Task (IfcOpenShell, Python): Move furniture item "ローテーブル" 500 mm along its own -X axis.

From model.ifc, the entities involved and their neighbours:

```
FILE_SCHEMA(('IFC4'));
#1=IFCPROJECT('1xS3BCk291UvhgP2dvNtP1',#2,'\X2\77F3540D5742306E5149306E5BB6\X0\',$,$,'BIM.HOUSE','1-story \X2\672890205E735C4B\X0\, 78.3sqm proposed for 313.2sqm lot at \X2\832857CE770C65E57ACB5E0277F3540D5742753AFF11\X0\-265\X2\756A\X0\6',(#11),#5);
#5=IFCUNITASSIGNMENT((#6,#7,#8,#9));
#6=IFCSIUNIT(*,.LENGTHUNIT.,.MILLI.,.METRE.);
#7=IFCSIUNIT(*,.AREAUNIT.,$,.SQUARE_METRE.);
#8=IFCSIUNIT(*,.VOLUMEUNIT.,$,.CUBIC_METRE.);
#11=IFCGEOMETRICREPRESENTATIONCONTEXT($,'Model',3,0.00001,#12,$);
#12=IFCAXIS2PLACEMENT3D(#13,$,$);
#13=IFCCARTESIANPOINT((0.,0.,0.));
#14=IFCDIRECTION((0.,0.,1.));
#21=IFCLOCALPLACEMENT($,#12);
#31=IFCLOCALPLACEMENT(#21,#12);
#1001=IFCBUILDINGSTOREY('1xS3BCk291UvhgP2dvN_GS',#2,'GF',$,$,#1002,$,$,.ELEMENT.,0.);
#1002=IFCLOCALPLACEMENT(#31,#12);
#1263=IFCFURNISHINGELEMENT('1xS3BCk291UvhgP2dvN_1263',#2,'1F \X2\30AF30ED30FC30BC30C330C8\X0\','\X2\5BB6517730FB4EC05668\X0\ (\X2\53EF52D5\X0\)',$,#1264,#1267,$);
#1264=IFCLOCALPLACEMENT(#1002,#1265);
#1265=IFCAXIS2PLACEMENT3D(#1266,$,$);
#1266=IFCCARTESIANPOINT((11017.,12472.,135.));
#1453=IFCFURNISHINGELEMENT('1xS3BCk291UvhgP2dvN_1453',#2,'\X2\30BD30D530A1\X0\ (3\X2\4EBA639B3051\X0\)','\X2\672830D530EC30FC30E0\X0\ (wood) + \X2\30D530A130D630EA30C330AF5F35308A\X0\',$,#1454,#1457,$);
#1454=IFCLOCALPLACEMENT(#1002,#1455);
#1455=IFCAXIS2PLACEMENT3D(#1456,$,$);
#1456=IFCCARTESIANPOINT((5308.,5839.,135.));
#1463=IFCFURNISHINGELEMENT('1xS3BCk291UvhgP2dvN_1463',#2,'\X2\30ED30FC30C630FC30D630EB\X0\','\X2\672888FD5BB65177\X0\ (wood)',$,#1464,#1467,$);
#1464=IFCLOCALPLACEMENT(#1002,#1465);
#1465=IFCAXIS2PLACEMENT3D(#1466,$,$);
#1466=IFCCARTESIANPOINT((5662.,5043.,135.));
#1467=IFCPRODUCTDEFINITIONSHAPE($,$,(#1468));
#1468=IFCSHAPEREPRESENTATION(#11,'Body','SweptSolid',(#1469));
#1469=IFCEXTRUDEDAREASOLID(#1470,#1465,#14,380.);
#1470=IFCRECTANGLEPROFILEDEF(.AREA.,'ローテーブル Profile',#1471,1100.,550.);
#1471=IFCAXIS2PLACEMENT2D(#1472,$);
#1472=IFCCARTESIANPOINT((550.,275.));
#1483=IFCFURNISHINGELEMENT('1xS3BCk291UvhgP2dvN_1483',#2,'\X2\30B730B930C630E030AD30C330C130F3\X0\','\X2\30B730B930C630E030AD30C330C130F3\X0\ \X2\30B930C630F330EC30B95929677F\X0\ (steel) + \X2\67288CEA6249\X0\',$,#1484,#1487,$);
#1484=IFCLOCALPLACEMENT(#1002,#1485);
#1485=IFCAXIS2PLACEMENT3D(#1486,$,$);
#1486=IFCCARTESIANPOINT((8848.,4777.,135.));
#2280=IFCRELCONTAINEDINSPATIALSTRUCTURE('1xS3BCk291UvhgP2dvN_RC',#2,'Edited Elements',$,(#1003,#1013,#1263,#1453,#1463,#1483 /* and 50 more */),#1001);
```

```python
import ifcopenshell
import ifcopenshell.api.geometry
import ifcopenshell.util.placement
import ifcopenshell.util.unit

model = ifcopenshell.open("model.ifc")
unit_scale = ifcopenshell.util.unit.calculate_unit_scale(model)

item = model.by_guid("1xS3BCk291UvhgP2dvN_1463")
matrix = ifcopenshell.util.placement.get_local_placement(item.ObjectPlacement)
matrix[:3, 3] -= matrix[:3, 0] * 0.5 / unit_scale
ifcopenshell.api.geometry.edit_object_placement(model, product=item, matrix=matrix, is_si=False)

print(ifcopenshell.util.placement.get_local_placement(item.ObjectPlacement).round(3) + 0.0)

model.write("model_edited.ifc")
```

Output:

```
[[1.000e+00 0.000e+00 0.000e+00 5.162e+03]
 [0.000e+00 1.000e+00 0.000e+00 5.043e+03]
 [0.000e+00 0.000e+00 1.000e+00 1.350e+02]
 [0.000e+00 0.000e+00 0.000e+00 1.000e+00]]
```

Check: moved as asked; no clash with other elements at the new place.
